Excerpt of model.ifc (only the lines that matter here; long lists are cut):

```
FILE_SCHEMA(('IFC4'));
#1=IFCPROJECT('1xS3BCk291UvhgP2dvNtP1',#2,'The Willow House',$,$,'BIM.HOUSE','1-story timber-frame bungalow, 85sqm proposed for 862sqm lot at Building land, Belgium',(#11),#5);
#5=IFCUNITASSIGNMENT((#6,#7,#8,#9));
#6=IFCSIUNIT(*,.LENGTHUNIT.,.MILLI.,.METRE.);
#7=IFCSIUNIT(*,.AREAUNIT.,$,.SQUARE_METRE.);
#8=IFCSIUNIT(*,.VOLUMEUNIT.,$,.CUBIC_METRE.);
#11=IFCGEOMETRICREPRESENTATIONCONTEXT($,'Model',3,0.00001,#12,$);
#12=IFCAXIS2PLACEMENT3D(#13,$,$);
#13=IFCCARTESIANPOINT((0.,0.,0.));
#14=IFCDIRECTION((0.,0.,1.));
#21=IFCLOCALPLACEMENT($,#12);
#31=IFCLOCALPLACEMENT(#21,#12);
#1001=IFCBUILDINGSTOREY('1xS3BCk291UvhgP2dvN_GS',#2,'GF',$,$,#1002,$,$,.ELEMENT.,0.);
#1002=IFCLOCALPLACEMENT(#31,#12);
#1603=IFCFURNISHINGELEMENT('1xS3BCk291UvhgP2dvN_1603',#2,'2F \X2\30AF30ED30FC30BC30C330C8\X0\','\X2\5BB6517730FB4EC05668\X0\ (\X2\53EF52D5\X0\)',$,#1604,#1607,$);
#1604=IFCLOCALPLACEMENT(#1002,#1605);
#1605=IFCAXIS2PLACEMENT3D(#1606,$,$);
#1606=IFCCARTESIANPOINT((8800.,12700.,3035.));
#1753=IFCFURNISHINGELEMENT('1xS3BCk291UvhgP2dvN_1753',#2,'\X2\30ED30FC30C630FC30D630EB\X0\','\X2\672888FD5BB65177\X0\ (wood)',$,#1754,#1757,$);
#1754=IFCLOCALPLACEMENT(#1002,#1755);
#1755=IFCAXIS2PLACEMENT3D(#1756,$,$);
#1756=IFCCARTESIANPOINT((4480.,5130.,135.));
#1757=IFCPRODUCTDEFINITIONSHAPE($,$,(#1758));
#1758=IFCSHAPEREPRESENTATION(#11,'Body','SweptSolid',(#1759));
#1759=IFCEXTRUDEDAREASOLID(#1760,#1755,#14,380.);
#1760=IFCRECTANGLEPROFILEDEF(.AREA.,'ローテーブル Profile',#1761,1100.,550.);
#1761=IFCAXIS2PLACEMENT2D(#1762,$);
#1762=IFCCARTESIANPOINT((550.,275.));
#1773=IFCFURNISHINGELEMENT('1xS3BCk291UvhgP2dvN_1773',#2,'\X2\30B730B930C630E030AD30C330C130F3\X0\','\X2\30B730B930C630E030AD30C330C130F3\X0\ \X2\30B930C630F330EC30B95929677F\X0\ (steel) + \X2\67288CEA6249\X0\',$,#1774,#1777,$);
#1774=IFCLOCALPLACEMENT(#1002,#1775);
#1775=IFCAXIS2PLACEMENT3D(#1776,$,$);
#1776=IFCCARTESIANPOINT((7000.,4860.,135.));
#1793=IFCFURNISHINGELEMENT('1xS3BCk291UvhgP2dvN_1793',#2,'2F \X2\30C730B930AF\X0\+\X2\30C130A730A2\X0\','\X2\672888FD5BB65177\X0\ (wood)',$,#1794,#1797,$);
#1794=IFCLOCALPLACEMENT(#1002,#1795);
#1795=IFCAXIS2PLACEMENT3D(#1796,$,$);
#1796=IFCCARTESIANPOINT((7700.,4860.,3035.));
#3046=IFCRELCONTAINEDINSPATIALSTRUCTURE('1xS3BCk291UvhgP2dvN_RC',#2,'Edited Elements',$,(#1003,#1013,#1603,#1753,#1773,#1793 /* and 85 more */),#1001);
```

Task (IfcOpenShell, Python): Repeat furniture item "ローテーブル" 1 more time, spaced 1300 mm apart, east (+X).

```python
import numpy as np
import ifcopenshell
import ifcopenshell.api.geometry
import ifcopenshell.api.root
import ifcopenshell.util.element
import ifcopenshell.util.placement
import ifcopenshell.util.unit

model = ifcopenshell.open("model.ifc")
unit_scale = ifcopenshell.util.unit.calculate_unit_scale(model)


def reuse_history(source, copy):
    """copy_class also copies each property set's owner history, people and application; keep the originals."""
    for rel in copy.IsDefinedBy:
        if rel.is_a("IfcRelDefinesByProperties") and (history := rel.RelatingPropertyDefinition.OwnerHistory):
            rel.RelatingPropertyDefinition.OwnerHistory = source.OwnerHistory
            ifcopenshell.util.element.remove_deep2(model, history)


source = model.by_guid("1xS3BCk291UvhgP2dvN_1753")
base = ifcopenshell.util.placement.get_local_placement(source.ObjectPlacement)
step = np.array([1.0, 0.0, 0.0]) * 1.3 / unit_scale

for i in range(1, 2):
    copy = ifcopenshell.api.root.copy_class(model, product=source)
    copy.Representation = ifcopenshell.util.element.copy_deep(
        model, source.Representation, exclude=["IfcGeometricRepresentationContext", "IfcRepresentationMap"]
    )
    reuse_history(source, copy)
    matrix = base.copy()
    matrix[:3, 3] += i * step
    print("added at", matrix[:3, 3].round(3) + 0.0)
    ifcopenshell.api.geometry.edit_object_placement(model, product=copy, matrix=matrix, is_si=False)

model.write("model_v2.ifc")
```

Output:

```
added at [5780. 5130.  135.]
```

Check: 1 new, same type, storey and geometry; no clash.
